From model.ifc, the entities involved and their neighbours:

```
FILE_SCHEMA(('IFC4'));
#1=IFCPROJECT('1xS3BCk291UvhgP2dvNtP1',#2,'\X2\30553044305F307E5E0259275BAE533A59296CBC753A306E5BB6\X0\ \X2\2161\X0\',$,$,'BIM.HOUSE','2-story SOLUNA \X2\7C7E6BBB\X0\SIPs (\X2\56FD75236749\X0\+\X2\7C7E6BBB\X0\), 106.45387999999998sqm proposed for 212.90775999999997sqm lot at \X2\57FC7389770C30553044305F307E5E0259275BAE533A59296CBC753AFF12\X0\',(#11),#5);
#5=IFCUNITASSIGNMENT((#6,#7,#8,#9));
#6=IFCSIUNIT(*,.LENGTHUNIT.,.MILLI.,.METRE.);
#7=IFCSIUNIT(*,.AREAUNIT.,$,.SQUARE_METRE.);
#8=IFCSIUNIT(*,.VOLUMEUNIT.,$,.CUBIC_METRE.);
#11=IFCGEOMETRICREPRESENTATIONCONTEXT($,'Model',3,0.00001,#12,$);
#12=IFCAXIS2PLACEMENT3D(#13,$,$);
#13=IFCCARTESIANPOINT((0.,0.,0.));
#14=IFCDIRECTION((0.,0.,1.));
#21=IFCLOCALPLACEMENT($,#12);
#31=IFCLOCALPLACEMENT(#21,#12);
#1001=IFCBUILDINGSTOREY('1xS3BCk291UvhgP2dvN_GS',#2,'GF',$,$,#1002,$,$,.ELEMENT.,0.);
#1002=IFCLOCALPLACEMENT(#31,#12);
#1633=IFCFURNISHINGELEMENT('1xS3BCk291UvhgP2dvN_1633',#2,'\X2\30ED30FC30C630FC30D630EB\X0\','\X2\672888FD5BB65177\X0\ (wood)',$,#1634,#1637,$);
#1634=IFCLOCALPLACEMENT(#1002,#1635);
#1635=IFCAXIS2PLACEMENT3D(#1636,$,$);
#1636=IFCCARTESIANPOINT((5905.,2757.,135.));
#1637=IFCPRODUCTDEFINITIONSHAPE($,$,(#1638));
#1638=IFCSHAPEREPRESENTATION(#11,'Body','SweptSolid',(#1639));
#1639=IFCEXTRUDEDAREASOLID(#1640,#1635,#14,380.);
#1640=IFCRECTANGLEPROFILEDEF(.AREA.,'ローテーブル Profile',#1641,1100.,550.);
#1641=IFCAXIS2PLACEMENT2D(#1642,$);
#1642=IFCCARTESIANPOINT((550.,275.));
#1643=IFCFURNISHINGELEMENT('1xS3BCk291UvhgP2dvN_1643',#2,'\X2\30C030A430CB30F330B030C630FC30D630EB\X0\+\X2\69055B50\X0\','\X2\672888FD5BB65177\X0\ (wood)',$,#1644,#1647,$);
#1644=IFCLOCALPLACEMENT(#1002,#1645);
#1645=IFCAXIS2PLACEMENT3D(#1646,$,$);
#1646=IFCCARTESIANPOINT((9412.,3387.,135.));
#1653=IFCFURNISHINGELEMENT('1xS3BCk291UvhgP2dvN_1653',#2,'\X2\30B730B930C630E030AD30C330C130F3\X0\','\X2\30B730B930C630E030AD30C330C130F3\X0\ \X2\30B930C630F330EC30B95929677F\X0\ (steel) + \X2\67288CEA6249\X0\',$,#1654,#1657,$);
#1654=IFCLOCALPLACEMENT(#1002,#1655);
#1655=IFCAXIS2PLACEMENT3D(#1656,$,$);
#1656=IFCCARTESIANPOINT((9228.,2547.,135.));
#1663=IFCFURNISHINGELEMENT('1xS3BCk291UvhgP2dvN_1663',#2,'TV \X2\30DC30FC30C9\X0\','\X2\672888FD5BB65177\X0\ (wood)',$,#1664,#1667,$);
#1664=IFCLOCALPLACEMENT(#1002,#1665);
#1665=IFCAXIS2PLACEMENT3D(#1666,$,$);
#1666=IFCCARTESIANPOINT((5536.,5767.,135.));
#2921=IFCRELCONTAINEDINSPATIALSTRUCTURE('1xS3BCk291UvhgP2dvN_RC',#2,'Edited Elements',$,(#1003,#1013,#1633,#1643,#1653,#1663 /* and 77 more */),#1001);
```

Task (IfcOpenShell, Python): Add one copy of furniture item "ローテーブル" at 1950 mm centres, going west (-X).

```python
import numpy as np
import ifcopenshell
import ifcopenshell.api.geometry
import ifcopenshell.api.root
import ifcopenshell.util.element
import ifcopenshell.util.placement

model = ifcopenshell.open("model.ifc")


def reuse_history(source, copy):
    """copy_class also copies each property set's owner history, people and application; keep the originals."""
    for rel in copy.IsDefinedBy:
        if rel.is_a("IfcRelDefinesByProperties") and (history := rel.RelatingPropertyDefinition.OwnerHistory):
            rel.RelatingPropertyDefinition.OwnerHistory = source.OwnerHistory
            ifcopenshell.util.element.remove_deep2(model, history)


source = model.by_id(1633)
base = ifcopenshell.util.placement.get_local_placement(source.ObjectPlacement)
step = np.array([-1.0, 0.0, 0.0]) * 1950.0

for i in range(1, 2):
    copy = ifcopenshell.api.root.copy_class(model, product=source)
    copy.Representation = ifcopenshell.util.element.copy_deep(
        model, source.Representation, exclude=["IfcGeometricRepresentationContext", "IfcRepresentationMap"]
    )
    reuse_history(source, copy)
    matrix = base.copy()
    matrix[:3, 3] += i * step
    print("added at", matrix[:3, 3].round(3) + 0.0)
    ifcopenshell.api.geometry.edit_object_placement(model, product=copy, matrix=matrix, is_si=False)

model.write("model_updated.ifc")
```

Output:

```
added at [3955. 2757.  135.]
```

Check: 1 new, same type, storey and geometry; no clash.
